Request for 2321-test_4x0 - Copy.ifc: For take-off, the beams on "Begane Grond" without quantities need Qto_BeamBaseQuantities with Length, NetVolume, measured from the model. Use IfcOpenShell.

First a look at what the model holds.

```python
import ifcopenshell
import ifcopenshell.util.element
import ifcopenshell.util.unit

model = ifcopenshell.open("2321-test_4x0 - Copy.ifc")
print(model.schema)
for unit_type in ("LENGTHUNIT", "AREAUNIT", "VOLUMEUNIT"):
    print(unit_type, ifcopenshell.util.unit.calculate_unit_scale(model, unit_type))
storey = next(s for s in model.by_type("IfcBuildingStorey") if s.Name == "Begane Grond")
beams = [e for e in ifcopenshell.util.element.get_decomposition(storey) if e.is_a("IfcBeam")]
for e in sorted(beams, key=lambda e: e.id()):
    print(e.id(), e.is_a(), e.Name, list(ifcopenshell.util.element.get_psets(e, qtos_only=True)), sep=" | ")
```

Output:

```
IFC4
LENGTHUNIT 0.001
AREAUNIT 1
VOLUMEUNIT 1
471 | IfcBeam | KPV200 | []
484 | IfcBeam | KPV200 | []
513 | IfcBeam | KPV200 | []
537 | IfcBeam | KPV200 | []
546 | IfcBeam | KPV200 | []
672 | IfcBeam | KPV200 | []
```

```python
import ifcopenshell
import ifcopenshell.api.pset
import ifcopenshell.geom
import ifcopenshell.util.element
import ifcopenshell.util.shape
import ifcopenshell.util.unit

model = ifcopenshell.open("2321-test_4x0 - Copy.ifc")
unit_scale = ifcopenshell.util.unit.calculate_unit_scale(model)
volume_scale = ifcopenshell.util.unit.calculate_unit_scale(model, "VOLUMEUNIT")
settings = ifcopenshell.geom.settings()

storey = next(s for s in model.by_type("IfcBuildingStorey") if s.Name == "Begane Grond")
beams = [e for e in ifcopenshell.util.element.get_decomposition(storey) if e.is_a("IfcBeam")]

for e in sorted(beams, key=lambda e: e.id()):
    if ifcopenshell.util.element.get_psets(e, qtos_only=True, should_inherit=False):
        continue
    # Geometry comes back in metres, in the element's own axes.
    shape = ifcopenshell.geom.create_shape(settings, e)
    values = {
        "Length": ifcopenshell.util.shape.get_max_xyz(shape.geometry) / unit_scale,
        "NetVolume": ifcopenshell.util.shape.get_volume(shape.geometry) / volume_scale,
    }
    qto = ifcopenshell.api.pset.add_qto(model, product=e, name="Qto_BeamBaseQuantities")
    ifcopenshell.api.pset.edit_qto(model, qto=qto, properties=values)
    print(e.id(), {k: round(v, 3) for k, v in values.items()})

model.write("2321-test_4x0 - Copy_updated.ifc")
```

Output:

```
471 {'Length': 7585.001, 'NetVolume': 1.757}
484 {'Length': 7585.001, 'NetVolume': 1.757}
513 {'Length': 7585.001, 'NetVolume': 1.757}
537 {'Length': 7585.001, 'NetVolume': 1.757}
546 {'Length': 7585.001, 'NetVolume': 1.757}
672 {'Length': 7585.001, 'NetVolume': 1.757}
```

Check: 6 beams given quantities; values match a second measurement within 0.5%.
